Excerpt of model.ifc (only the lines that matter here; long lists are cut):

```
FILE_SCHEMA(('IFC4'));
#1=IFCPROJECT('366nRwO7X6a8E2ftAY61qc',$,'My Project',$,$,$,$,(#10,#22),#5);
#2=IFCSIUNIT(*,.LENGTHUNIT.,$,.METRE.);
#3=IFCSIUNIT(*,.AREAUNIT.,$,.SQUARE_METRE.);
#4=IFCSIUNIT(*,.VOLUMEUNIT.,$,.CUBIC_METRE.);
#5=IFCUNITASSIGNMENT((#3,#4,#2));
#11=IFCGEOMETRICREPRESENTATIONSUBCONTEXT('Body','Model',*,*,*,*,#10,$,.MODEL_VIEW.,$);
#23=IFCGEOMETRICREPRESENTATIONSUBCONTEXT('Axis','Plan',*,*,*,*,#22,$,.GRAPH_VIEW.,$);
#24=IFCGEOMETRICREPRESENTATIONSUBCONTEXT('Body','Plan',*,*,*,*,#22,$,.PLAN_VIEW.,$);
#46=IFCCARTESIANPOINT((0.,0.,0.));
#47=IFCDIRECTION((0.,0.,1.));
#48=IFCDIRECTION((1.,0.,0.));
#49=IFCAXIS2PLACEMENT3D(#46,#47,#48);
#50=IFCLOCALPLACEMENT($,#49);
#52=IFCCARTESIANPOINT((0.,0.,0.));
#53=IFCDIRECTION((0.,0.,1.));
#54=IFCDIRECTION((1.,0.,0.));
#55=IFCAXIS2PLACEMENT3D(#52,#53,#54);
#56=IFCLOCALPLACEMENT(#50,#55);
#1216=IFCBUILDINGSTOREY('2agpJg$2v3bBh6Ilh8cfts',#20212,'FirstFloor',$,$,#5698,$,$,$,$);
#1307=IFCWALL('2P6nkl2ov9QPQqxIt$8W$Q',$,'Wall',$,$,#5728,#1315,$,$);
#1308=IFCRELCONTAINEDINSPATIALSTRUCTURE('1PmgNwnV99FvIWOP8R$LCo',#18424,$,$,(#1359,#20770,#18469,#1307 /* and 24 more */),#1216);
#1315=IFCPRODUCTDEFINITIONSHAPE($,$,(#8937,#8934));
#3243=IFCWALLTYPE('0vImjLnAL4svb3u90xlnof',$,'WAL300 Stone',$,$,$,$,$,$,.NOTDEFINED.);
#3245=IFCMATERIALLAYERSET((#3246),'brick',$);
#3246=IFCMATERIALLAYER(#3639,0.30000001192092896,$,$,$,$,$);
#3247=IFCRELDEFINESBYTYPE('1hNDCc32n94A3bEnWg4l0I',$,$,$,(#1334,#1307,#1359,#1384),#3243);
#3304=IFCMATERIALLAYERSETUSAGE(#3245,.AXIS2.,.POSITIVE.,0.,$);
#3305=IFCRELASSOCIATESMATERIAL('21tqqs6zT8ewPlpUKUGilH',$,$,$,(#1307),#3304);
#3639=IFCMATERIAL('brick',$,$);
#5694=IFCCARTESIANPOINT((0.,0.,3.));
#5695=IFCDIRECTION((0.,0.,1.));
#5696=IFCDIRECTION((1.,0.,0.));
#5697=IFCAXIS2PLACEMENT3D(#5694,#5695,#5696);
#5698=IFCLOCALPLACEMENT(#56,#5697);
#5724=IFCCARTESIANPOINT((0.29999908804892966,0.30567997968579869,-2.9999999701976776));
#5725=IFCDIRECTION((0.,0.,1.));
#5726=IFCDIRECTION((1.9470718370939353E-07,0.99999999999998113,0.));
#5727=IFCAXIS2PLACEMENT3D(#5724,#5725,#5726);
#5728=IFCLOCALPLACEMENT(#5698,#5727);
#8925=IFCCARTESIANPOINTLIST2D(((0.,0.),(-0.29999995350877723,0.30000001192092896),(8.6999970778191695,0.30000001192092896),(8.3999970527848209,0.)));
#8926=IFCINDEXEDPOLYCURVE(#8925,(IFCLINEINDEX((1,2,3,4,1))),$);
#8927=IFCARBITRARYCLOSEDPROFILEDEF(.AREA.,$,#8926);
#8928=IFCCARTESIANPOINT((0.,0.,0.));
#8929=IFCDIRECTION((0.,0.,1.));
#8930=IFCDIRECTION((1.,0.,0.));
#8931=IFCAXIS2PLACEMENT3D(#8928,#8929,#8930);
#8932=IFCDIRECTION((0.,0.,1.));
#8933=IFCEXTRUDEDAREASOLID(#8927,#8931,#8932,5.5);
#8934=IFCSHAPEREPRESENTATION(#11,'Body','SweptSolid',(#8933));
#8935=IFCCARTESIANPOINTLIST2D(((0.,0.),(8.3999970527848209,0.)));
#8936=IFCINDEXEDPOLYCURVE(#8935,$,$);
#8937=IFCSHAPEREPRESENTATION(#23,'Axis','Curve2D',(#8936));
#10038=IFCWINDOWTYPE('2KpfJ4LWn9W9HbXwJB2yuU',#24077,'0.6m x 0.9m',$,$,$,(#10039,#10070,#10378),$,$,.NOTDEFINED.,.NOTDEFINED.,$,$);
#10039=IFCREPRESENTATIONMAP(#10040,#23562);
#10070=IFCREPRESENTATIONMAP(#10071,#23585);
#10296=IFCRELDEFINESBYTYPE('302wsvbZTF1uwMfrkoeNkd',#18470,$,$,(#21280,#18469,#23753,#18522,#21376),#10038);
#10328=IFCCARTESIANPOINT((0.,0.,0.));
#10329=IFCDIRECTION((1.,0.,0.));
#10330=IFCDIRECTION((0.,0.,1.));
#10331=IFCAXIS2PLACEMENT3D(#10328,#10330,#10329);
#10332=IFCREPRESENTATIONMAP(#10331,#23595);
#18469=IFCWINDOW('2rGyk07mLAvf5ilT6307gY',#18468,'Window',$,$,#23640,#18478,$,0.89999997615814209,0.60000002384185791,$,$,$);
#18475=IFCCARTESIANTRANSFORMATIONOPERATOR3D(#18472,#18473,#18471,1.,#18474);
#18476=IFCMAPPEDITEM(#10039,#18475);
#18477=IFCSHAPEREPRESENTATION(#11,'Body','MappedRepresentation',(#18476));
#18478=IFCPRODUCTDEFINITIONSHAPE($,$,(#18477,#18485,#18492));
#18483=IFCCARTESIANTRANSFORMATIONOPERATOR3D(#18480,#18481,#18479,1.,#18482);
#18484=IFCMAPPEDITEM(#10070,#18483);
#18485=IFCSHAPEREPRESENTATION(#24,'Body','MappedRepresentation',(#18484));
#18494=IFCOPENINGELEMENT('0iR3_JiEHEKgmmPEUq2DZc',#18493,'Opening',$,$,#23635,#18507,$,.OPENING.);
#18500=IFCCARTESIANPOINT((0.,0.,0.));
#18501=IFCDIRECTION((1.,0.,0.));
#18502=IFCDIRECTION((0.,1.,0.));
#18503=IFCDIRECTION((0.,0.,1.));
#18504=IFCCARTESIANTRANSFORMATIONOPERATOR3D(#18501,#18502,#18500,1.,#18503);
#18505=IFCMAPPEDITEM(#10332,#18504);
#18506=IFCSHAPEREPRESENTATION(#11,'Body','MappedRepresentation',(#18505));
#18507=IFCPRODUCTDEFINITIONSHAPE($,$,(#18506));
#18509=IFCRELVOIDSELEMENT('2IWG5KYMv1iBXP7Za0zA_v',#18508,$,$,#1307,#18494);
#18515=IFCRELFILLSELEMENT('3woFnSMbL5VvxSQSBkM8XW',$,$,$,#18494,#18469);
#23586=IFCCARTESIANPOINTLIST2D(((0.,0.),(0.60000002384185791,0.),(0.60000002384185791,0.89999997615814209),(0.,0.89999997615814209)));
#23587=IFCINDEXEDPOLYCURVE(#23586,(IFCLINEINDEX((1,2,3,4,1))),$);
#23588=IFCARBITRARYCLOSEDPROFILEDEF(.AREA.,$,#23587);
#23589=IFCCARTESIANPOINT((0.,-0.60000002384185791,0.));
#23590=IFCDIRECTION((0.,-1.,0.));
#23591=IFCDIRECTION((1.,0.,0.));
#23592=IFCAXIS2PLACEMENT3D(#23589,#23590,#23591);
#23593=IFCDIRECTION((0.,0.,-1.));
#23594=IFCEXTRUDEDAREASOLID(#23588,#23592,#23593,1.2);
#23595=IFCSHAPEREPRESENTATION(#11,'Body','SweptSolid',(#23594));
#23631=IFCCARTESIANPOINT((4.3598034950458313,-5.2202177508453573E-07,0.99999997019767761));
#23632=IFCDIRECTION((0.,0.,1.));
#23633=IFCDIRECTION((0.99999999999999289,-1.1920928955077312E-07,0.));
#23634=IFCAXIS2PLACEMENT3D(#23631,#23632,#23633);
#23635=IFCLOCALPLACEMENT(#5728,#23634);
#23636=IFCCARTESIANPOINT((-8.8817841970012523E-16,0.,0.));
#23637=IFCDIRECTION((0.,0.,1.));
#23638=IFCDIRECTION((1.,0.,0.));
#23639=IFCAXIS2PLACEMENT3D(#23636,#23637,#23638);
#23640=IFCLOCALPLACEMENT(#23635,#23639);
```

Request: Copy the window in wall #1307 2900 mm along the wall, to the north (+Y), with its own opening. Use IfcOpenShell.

```python
import ifcopenshell
import ifcopenshell.api.feature
import ifcopenshell.api.geometry
import ifcopenshell.api.root
import ifcopenshell.geom
import ifcopenshell.util.element
import ifcopenshell.util.placement
import ifcopenshell.util.shape

model = ifcopenshell.open("model.ifc")
settings = ifcopenshell.geom.settings()


def volume(element):
    """Net volume in cubic metres, openings subtracted."""
    shape = ifcopenshell.geom.create_shape(settings, element)
    return ifcopenshell.util.shape.get_volume(shape.geometry)


window = model.by_id(18469)
opening = window.FillsVoids[0].RelatingOpeningElement
wall = opening.VoidsElements[0].RelatingBuildingElement
before = volume(wall)
shift = ifcopenshell.util.placement.get_local_placement(wall.ObjectPlacement)[:3, 0] * 2.9

# copy_class copies the void relationship, type, container and properties, but no geometry.
new_opening = ifcopenshell.api.root.copy_class(model, product=opening)
new_opening.Representation = ifcopenshell.util.element.copy_deep(
    model, opening.Representation, exclude=["IfcGeometricRepresentationContext", "IfcRepresentationMap"]
)
new_window = ifcopenshell.api.root.copy_class(model, product=window)
new_window.Representation = ifcopenshell.util.element.copy_deep(
    model, window.Representation, exclude=["IfcGeometricRepresentationContext", "IfcRepresentationMap"]
)
ifcopenshell.api.feature.add_filling(model, opening=new_opening, element=new_window)

for old, new in ((opening, new_opening), (window, new_window)):
    matrix = ifcopenshell.util.placement.get_local_placement(old.ObjectPlacement)
    matrix[:3, 3] += shift
    ifcopenshell.api.geometry.edit_object_placement(model, product=new, matrix=matrix, is_si=False)

after = volume(wall)

print(f"wall volume {before:.3f} -> {after:.3f} m3")

model.write("model_updated.ifc")
```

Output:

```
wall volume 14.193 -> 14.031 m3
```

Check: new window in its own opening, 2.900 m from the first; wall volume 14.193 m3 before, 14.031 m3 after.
